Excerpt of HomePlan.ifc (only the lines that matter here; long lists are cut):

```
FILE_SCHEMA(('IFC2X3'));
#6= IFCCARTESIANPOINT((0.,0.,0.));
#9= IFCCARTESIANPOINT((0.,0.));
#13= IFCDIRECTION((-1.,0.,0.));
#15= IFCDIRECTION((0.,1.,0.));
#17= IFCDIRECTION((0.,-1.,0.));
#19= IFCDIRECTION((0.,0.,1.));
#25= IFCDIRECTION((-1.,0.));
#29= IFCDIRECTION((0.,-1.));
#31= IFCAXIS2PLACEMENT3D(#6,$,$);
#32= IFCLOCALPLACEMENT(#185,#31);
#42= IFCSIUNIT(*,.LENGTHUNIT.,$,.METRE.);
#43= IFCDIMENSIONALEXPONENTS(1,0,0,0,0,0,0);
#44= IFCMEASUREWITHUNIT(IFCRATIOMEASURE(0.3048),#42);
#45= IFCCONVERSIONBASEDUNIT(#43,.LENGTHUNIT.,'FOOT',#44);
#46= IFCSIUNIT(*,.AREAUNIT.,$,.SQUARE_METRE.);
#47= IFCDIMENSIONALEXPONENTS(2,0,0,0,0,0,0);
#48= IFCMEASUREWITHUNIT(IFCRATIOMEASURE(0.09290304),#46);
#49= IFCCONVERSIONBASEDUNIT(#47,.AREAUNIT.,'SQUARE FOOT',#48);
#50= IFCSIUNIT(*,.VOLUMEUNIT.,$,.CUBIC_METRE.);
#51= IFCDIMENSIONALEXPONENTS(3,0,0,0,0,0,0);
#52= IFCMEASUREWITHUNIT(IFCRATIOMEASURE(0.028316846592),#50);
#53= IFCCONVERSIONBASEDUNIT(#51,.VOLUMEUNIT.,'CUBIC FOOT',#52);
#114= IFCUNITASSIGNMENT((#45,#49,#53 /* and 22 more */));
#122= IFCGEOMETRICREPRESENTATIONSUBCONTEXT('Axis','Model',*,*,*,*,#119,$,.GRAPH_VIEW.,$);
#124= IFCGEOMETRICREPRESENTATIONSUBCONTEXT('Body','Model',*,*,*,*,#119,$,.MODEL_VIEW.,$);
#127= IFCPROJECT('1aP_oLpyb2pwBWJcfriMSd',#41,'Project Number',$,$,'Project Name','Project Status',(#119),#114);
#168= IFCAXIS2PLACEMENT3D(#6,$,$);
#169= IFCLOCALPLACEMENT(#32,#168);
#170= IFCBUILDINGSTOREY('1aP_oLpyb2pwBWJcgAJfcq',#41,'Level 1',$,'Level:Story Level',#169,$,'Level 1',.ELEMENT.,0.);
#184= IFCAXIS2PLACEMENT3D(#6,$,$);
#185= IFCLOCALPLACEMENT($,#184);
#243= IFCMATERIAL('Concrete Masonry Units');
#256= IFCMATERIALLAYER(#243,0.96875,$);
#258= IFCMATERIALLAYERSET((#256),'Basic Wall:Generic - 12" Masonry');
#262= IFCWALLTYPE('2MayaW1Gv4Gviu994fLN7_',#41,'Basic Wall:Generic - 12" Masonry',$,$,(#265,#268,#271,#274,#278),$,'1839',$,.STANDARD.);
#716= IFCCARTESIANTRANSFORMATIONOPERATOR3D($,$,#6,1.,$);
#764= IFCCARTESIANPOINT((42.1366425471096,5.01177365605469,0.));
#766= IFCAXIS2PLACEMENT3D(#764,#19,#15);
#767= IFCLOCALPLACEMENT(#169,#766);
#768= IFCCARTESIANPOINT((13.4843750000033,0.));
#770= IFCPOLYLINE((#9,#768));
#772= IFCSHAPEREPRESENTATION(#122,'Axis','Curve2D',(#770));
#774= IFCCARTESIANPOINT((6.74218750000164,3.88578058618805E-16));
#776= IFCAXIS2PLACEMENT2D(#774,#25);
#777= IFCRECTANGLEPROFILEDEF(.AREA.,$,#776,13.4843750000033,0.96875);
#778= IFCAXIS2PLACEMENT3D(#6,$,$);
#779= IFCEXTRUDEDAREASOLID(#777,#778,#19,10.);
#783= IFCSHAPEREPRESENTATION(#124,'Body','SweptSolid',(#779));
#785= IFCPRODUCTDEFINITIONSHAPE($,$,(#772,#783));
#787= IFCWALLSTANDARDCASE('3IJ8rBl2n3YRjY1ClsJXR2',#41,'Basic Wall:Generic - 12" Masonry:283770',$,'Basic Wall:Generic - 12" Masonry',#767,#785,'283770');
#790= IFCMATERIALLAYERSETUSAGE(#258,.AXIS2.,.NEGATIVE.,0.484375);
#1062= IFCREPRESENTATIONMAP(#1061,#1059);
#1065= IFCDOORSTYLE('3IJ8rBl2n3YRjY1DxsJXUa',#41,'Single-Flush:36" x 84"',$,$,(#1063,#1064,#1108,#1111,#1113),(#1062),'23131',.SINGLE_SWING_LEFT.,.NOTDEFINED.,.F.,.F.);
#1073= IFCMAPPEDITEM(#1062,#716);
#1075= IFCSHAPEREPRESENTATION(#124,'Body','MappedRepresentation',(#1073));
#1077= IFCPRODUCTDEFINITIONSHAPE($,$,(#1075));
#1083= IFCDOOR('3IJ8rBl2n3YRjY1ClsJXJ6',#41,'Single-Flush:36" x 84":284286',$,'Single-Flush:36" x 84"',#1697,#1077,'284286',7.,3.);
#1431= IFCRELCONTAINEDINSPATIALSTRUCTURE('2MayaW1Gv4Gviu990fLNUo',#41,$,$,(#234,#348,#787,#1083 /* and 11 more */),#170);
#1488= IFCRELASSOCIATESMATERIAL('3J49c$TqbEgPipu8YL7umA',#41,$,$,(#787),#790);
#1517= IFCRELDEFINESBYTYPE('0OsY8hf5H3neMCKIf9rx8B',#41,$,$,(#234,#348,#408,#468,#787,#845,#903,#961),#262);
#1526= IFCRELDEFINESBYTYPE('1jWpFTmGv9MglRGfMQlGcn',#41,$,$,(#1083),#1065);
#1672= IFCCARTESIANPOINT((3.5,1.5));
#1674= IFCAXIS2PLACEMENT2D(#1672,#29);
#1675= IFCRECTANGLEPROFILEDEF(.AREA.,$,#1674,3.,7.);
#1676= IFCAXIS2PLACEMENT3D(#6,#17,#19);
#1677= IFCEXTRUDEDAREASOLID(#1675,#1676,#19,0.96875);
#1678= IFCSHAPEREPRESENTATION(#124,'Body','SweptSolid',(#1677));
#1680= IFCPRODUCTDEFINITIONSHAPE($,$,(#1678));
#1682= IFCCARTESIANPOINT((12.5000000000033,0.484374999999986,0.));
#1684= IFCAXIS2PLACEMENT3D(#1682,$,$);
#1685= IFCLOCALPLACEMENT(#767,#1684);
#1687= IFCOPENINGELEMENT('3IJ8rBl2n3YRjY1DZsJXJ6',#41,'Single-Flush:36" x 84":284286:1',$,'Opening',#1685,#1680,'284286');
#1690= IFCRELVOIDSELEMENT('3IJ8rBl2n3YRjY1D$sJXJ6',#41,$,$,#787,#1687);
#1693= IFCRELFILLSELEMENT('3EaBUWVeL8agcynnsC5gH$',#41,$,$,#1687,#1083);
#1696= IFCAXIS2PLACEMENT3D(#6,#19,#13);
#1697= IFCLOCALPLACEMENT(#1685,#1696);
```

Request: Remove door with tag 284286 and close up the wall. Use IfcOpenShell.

```python
import ifcopenshell
import ifcopenshell.api.feature
import ifcopenshell.api.root
import ifcopenshell.geom
import ifcopenshell.util.shape

model = ifcopenshell.open("HomePlan.ifc")
settings = ifcopenshell.geom.settings()


def volume(element):
    """Net volume in cubic metres, openings subtracted."""
    shape = ifcopenshell.geom.create_shape(settings, element)
    return ifcopenshell.util.shape.get_volume(shape.geometry)


door = model.by_id(1083)
opening = door.FillsVoids[0].RelatingOpeningElement
wall = opening.VoidsElements[0].RelatingBuildingElement
before = volume(wall)

ifcopenshell.api.root.remove_product(model, product=door)
ifcopenshell.api.feature.remove_feature(model, feature=opening)

after = volume(wall)

print(f"wall volume {before:.3f} -> {after:.3f} m3")

model.write("HomePlan-out.ifc")
```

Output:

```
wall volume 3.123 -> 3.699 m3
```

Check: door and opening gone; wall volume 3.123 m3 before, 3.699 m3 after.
